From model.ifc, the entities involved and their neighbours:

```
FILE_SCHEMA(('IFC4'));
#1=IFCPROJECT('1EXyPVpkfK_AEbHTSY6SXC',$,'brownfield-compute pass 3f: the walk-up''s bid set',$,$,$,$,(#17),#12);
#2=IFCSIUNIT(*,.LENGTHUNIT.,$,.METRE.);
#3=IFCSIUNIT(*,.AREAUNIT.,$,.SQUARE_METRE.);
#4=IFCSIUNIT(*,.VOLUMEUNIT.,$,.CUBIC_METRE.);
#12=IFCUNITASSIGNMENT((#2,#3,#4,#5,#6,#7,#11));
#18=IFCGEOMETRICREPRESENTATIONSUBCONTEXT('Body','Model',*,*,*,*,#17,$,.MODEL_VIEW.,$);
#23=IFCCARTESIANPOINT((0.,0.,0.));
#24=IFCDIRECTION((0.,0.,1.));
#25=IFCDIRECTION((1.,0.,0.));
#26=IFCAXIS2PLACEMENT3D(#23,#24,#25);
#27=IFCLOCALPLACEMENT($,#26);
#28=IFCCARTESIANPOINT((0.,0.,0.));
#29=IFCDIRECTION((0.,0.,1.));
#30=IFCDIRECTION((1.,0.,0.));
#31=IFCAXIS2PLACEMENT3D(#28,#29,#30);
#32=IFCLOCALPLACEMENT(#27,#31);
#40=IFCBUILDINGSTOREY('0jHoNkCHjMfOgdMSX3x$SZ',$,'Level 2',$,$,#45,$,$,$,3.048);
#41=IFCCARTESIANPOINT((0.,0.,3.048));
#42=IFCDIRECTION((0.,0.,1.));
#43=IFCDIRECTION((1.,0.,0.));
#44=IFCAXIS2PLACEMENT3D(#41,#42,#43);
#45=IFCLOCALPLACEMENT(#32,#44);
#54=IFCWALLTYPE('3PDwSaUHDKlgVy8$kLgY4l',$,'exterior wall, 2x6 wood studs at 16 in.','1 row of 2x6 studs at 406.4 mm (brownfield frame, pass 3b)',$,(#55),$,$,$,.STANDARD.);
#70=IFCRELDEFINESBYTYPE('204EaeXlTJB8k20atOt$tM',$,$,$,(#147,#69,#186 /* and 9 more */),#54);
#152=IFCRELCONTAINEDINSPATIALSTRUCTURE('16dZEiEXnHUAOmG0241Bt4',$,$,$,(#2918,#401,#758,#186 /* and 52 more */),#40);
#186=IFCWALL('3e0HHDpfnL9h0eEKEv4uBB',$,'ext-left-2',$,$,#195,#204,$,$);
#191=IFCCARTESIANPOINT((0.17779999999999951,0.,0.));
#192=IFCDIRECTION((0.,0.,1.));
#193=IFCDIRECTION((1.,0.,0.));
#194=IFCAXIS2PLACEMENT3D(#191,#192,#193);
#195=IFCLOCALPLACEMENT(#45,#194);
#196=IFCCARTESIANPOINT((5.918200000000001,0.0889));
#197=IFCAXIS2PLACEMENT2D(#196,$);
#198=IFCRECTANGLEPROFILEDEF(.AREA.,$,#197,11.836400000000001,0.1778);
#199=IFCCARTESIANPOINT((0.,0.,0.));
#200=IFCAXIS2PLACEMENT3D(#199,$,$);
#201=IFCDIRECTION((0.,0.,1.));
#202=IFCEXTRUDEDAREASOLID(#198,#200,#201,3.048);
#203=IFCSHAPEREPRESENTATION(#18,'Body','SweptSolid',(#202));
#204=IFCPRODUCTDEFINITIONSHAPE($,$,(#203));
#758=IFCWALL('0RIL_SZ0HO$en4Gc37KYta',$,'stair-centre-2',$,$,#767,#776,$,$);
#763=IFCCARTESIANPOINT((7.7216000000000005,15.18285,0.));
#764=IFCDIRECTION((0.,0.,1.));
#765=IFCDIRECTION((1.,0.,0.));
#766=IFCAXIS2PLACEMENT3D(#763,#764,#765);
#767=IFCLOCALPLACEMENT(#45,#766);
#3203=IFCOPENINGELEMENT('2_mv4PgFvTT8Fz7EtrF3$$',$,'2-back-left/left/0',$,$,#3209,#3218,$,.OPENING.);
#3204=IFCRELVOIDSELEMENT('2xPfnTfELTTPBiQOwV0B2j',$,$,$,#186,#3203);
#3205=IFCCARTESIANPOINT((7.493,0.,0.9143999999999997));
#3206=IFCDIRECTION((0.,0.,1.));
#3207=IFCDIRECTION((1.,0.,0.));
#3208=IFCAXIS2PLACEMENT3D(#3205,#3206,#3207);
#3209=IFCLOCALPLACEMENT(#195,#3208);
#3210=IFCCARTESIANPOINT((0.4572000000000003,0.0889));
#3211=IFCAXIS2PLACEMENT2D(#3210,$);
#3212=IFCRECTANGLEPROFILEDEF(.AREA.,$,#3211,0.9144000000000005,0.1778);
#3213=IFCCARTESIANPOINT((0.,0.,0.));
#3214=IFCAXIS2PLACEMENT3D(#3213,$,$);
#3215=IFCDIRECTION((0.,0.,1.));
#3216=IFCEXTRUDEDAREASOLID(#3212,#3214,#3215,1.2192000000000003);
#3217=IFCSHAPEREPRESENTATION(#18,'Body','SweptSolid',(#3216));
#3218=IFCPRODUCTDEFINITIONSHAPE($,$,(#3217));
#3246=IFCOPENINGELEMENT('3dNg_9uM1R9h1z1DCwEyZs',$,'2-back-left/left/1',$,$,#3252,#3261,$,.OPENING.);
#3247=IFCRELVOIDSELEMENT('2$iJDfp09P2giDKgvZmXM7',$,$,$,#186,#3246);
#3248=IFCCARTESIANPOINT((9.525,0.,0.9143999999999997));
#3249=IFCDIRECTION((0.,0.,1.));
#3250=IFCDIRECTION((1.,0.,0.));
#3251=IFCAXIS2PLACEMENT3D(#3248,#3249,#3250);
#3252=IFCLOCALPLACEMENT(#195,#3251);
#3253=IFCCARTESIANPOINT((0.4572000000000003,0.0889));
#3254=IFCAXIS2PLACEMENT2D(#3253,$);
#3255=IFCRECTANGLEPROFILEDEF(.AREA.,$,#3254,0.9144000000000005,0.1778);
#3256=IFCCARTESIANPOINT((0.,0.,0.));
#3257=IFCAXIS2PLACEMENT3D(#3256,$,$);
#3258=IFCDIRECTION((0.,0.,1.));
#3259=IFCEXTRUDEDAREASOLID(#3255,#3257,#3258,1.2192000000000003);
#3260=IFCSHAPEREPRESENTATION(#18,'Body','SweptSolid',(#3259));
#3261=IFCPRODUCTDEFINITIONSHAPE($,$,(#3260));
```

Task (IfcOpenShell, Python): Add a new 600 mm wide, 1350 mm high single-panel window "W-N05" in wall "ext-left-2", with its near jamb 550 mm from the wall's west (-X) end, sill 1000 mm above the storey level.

```python
import numpy as np
import ifcopenshell
import ifcopenshell.api.feature
import ifcopenshell.api.geometry
import ifcopenshell.api.root
import ifcopenshell.api.spatial
import ifcopenshell.geom
import ifcopenshell.util.element
import ifcopenshell.util.placement
import ifcopenshell.util.representation
import ifcopenshell.util.shape
import ifcopenshell.util.unit

model = ifcopenshell.open("model.ifc")
unit_scale = ifcopenshell.util.unit.calculate_unit_scale(model)
settings = ifcopenshell.geom.settings()


def volume(element):
    """Net volume in cubic metres, openings subtracted."""
    shape = ifcopenshell.geom.create_shape(settings, element)
    return ifcopenshell.util.shape.get_volume(shape.geometry)


wall = model.by_id(186)
storey = ifcopenshell.util.element.get_container(wall, ifc_class="IfcBuildingStorey")
context = ifcopenshell.util.representation.get_context(model, "Model", "Body", "MODEL_VIEW")
before = volume(wall)

width, height, from_end, sill = 0.6, 1.35, 0.55, 1  # metres

# The wall runs along its own X axis, and the end named is its -X end.
wall_shape = ifcopenshell.geom.create_shape(settings, wall)
x, y, z = ifcopenshell.util.shape.get_vertices(wall_shape.geometry).T
start = x.min() + from_end
face, thickness = float(y.min()), float(y.max() - y.min())
wall_matrix = ifcopenshell.util.placement.get_local_placement(wall.ObjectPlacement)
level = ifcopenshell.util.placement.get_local_placement(storey.ObjectPlacement)[2, 3]


def in_wall(x, y):
    """Placement at x, y metres in the wall's axes, at sill height."""
    matrix = wall_matrix.copy()
    matrix[:, 3] = wall_matrix @ np.array([x / unit_scale, y / unit_scale, 0.0, 1.0])
    matrix[2, 3] = level + sill / unit_scale
    return matrix


# Opening: a box that overshoots both wall faces by 50 mm.
opening = ifcopenshell.api.root.create_entity(model, ifc_class="IfcOpeningElement", predefined_type="OPENING")
box = ifcopenshell.api.geometry.add_wall_representation(
    model, context=context, length=width, height=height, thickness=thickness + 0.1
)
ifcopenshell.api.geometry.assign_representation(model, product=opening, representation=box)
ifcopenshell.api.geometry.edit_object_placement(model, product=opening, matrix=in_wall(start, face - 0.05), is_si=False)
ifcopenshell.api.feature.add_feature(model, feature=opening, element=wall)

window = ifcopenshell.api.root.create_entity(model, ifc_class="IfcWindow", name="W-N05", predefined_type="WINDOW")
window.OverallWidth, window.OverallHeight = width / unit_scale, height / unit_scale
window.PartitioningType = "SINGLE_PANEL"
body = ifcopenshell.api.geometry.add_window_representation(
    model,
    context=context,
    overall_width=window.OverallWidth,
    overall_height=window.OverallHeight,
    partition_type="SINGLE_PANEL",
)
ifcopenshell.api.geometry.assign_representation(model, product=window, representation=body)
ifcopenshell.api.spatial.assign_container(model, products=[window], relating_structure=storey)
ifcopenshell.api.feature.add_filling(model, opening=opening, element=window)

# Centre the window in the wall's thickness.
ifcopenshell.api.geometry.edit_object_placement(model, product=window, matrix=in_wall(start, face), is_si=False)
window_shape = ifcopenshell.geom.create_shape(settings, window)
depth = ifcopenshell.util.shape.get_vertices(window_shape.geometry)[:, 1]
offset = face + thickness / 2 - (depth.min() + depth.max()) / 2
ifcopenshell.api.geometry.edit_object_placement(model, product=window, matrix=in_wall(start, offset), is_si=False)

after = volume(wall)

print(f"wall volume {before:.3f} -> {after:.3f} m3")

model.write("model_updated.ifc")
```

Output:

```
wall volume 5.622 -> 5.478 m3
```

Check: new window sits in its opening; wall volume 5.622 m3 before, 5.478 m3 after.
